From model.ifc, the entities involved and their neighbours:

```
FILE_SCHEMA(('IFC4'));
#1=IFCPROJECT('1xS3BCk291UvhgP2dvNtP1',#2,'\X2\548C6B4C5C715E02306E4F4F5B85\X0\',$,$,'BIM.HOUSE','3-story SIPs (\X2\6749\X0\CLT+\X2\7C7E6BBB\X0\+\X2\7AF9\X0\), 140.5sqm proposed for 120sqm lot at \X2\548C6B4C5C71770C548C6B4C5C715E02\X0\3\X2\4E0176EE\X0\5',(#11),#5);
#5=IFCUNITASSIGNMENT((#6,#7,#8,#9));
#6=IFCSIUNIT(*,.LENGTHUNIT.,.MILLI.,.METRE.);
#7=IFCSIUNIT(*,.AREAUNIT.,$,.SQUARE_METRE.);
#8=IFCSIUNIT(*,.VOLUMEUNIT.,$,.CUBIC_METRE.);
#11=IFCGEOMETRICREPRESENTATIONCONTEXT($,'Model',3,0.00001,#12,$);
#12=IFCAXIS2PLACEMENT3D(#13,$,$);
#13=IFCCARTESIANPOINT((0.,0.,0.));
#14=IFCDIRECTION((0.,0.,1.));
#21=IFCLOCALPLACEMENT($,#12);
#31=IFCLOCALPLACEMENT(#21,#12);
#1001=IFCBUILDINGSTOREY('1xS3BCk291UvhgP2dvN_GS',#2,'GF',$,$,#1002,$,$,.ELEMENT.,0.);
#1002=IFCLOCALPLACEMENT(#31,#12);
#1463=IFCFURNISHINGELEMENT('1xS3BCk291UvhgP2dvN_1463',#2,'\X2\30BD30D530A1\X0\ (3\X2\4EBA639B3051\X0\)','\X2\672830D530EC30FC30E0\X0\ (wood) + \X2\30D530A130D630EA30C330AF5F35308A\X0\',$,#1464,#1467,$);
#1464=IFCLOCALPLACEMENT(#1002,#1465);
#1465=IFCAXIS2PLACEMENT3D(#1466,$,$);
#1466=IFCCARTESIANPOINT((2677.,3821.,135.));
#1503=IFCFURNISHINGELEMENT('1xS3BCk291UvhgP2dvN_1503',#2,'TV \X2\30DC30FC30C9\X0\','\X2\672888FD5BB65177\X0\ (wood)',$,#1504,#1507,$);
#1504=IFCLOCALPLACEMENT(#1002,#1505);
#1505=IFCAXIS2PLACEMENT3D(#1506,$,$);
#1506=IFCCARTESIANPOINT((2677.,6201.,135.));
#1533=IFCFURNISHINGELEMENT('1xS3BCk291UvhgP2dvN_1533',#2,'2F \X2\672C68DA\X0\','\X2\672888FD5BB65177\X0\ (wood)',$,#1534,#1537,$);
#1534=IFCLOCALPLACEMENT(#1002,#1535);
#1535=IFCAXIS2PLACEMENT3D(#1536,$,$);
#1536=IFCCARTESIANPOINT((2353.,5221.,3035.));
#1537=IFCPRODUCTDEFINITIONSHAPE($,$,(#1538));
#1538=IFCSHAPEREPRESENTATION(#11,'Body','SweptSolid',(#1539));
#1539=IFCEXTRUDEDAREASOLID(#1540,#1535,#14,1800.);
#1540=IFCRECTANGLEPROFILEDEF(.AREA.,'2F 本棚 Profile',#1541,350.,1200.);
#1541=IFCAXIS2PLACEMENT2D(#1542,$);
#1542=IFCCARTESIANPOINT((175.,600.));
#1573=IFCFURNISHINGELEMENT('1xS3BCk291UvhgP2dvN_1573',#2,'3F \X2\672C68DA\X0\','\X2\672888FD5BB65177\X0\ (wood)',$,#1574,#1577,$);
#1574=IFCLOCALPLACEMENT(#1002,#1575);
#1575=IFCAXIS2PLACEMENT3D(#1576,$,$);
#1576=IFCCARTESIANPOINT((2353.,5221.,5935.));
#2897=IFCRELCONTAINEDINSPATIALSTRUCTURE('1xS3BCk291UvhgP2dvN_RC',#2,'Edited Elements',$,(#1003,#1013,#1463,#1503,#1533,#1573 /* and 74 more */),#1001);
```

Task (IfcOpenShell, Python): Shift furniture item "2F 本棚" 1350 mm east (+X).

```python
import ifcopenshell
import ifcopenshell.api.geometry
import ifcopenshell.util.placement
import ifcopenshell.util.unit

model = ifcopenshell.open("model.ifc")
unit_scale = ifcopenshell.util.unit.calculate_unit_scale(model)

item = model.by_guid("1xS3BCk291UvhgP2dvN_1533")
matrix = ifcopenshell.util.placement.get_local_placement(item.ObjectPlacement)
matrix[0, 3] += 1.35 / unit_scale
ifcopenshell.api.geometry.edit_object_placement(model, product=item, matrix=matrix, is_si=False)

print(ifcopenshell.util.placement.get_local_placement(item.ObjectPlacement).round(3) + 0.0)

model.write("model-out.ifc")
```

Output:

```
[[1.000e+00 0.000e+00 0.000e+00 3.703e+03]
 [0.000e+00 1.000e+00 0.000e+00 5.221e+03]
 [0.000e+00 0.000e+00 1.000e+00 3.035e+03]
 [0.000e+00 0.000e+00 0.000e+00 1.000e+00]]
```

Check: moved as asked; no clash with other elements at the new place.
